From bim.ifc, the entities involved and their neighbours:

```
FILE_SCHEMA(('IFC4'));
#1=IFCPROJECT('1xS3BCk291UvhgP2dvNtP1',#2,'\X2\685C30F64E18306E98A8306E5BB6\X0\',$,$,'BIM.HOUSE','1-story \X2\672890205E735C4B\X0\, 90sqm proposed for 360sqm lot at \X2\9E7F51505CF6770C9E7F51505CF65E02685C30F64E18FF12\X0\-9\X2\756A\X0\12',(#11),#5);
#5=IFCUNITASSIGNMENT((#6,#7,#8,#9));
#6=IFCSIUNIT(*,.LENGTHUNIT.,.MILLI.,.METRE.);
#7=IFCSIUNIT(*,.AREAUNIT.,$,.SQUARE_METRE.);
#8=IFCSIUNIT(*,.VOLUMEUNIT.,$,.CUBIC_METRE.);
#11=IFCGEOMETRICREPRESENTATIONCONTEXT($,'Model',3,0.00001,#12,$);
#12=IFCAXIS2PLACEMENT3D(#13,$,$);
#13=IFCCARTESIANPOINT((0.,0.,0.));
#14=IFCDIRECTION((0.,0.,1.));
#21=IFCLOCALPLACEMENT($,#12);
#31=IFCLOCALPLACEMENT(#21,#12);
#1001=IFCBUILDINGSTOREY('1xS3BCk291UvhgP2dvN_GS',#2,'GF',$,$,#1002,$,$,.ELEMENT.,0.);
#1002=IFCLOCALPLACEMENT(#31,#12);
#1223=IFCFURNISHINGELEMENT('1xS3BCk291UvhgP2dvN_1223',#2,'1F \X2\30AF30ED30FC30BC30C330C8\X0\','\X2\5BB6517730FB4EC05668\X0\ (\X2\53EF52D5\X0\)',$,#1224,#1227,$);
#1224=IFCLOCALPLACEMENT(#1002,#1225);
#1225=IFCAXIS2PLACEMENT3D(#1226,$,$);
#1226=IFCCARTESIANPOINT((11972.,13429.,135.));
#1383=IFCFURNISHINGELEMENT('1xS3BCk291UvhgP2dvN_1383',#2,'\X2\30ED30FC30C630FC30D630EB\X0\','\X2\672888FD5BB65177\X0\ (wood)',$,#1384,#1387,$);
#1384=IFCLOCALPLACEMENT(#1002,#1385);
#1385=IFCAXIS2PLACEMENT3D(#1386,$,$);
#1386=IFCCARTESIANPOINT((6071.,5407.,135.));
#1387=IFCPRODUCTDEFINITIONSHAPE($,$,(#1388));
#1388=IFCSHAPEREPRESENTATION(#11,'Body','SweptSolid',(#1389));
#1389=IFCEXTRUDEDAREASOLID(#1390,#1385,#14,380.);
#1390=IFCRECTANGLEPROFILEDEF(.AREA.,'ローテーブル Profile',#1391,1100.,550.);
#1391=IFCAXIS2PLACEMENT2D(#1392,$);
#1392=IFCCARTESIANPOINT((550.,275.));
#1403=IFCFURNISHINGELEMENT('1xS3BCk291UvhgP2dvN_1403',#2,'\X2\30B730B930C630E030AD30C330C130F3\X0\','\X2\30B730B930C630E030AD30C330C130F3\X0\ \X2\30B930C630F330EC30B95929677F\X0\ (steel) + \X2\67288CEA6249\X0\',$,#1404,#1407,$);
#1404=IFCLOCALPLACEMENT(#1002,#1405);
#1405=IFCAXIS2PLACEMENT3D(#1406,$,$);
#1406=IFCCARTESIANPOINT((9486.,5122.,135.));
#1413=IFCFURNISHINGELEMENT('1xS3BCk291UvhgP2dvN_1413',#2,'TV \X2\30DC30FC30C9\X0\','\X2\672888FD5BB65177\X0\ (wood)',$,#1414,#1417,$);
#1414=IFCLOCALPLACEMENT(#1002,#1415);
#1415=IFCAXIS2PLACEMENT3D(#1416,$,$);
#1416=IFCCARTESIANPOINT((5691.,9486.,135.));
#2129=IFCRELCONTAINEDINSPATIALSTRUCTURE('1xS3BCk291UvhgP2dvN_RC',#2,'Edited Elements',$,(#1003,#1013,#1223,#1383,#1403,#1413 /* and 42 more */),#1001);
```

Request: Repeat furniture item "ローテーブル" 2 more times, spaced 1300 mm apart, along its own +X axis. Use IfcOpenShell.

```python
import ifcopenshell
import ifcopenshell.api.geometry
import ifcopenshell.api.root
import ifcopenshell.util.element
import ifcopenshell.util.placement

model = ifcopenshell.open("bim.ifc")


def reuse_history(source, copy):
    """copy_class also copies each property set's owner history, people and application; keep the originals."""
    for rel in copy.IsDefinedBy:
        if rel.is_a("IfcRelDefinesByProperties") and (history := rel.RelatingPropertyDefinition.OwnerHistory):
            rel.RelatingPropertyDefinition.OwnerHistory = source.OwnerHistory
            ifcopenshell.util.element.remove_deep2(model, history)


source = model.by_id(1383)
base = ifcopenshell.util.placement.get_local_placement(source.ObjectPlacement)
step = base[:3, 0] * 1300.0

for i in range(1, 3):
    copy = ifcopenshell.api.root.copy_class(model, product=source)
    copy.Representation = ifcopenshell.util.element.copy_deep(
        model, source.Representation, exclude=["IfcGeometricRepresentationContext", "IfcRepresentationMap"]
    )
    reuse_history(source, copy)
    matrix = base.copy()
    matrix[:3, 3] += i * step
    print("added at", matrix[:3, 3].round(3) + 0.0)
    ifcopenshell.api.geometry.edit_object_placement(model, product=copy, matrix=matrix, is_si=False)

model.write("bim_edited.ifc")
```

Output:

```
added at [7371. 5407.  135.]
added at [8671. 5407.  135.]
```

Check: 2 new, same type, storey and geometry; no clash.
